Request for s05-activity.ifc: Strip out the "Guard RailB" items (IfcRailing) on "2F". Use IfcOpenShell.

First a look at what the model holds.

```python
import ifcopenshell
import ifcopenshell.util.element

model = ifcopenshell.open("s05-activity.ifc")
print(model.schema)
storey = next(s for s in model.by_type("IfcBuildingStorey") if s.Name == "2F")
railings = [e for e in ifcopenshell.util.element.get_decomposition(storey) if e.is_a("IfcRailing")]
seen = {}
for e in railings:
    element_type = ifcopenshell.util.element.get_type(e)
    name = element_type.Name if element_type not in (None, e) else None
    seen[name] = seen.get(name, 0) + 1
for name, count in sorted(seen.items(), key=str):
    print(count, "x", name)
```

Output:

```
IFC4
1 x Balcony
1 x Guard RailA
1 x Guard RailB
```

```python
import ifcopenshell
import ifcopenshell.api.root
import ifcopenshell.util.element

model = ifcopenshell.open("s05-activity.ifc")

storey = next(s for s in model.by_type("IfcBuildingStorey") if s.Name == "2F")
railings = [e for e in ifcopenshell.util.element.get_decomposition(storey) if e.is_a("IfcRailing")]
targets = [e for e in railings if (t := ifcopenshell.util.element.get_type(e)) not in (None, e) and t.Name == "Guard RailB"]

for e in targets:
    ifcopenshell.api.root.remove_product(model, product=e)
print(len(targets), "removed")

model.write("s05-activity_v2.ifc")
```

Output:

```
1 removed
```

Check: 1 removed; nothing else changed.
